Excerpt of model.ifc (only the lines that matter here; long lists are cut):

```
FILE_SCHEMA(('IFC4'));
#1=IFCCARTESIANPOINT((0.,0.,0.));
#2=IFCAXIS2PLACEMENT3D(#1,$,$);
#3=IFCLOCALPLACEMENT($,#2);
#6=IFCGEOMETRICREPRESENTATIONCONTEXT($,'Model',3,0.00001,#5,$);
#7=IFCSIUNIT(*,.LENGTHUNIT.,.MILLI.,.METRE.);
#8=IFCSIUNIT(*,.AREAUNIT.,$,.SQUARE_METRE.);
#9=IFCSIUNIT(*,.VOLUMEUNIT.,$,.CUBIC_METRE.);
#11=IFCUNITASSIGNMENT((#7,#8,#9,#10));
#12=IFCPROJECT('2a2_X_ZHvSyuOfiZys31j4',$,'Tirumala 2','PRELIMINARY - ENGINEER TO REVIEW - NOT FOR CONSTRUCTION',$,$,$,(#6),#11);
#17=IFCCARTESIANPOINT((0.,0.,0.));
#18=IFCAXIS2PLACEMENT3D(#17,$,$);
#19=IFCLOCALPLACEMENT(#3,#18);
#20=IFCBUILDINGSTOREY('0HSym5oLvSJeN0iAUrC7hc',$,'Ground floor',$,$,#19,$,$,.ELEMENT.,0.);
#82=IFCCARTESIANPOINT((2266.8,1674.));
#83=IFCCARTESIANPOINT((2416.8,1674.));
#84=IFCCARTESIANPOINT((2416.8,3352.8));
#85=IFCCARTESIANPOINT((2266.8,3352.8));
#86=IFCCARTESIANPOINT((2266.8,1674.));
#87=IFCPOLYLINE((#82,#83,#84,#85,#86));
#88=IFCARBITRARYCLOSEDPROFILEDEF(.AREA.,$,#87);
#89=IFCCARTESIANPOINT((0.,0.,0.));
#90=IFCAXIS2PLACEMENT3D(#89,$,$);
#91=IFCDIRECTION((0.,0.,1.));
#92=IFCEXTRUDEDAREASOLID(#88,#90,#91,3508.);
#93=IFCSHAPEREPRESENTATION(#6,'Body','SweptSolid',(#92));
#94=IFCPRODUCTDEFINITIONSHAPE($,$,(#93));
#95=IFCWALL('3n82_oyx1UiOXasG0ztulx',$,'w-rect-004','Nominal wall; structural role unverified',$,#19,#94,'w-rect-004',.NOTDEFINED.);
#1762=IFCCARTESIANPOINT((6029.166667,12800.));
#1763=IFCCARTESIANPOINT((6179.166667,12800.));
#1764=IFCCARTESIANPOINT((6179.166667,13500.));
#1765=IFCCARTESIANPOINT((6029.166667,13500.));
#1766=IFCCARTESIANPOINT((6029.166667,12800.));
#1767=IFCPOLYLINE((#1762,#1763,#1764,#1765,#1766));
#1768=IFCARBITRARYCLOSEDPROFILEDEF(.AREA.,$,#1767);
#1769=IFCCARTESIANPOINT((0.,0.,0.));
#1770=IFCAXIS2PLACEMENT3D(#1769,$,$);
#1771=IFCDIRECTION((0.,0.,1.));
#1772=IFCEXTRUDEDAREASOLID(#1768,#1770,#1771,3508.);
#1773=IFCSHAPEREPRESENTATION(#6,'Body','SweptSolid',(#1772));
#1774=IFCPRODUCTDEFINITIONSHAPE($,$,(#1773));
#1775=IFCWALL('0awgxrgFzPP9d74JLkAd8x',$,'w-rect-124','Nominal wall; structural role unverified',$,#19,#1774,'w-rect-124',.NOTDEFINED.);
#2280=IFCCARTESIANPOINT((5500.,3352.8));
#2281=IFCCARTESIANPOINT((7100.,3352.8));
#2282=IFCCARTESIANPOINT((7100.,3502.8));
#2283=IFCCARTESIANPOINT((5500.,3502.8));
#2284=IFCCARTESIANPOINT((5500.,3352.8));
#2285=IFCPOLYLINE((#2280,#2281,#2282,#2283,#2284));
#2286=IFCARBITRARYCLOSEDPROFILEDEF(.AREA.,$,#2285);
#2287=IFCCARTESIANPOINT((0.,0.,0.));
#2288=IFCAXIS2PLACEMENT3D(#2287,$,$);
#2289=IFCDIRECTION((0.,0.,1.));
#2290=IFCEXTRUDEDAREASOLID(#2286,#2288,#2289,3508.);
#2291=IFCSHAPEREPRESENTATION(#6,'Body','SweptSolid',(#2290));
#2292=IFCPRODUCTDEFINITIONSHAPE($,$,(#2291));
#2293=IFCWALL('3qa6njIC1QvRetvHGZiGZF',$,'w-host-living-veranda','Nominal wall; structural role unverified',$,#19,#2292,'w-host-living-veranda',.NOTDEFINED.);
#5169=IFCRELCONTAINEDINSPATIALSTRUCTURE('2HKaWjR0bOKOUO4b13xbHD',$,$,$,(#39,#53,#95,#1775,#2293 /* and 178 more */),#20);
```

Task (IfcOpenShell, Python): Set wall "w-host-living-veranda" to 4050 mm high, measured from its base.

```python
import ifcopenshell
import ifcopenshell.geom
import ifcopenshell.util.shape

model = ifcopenshell.open("model.ifc")
settings = ifcopenshell.geom.settings()


def volume(element):
    """Net volume in cubic metres, openings subtracted."""
    shape = ifcopenshell.geom.create_shape(settings, element)
    return ifcopenshell.util.shape.get_volume(shape.geometry)


wall = model.by_guid("3qa6njIC1QvRetvHGZiGZF")
before = volume(wall)

body = next(r for r in wall.Representation.Representations if r.RepresentationIdentifier == "Body")
solid = body.Items[0]
old_height = solid.Depth
solid.Depth = 4050.0
after = volume(wall)

print(f"height {old_height:g} -> {solid.Depth:g}, volume {before:.3f} -> {after:.3f} m3")

model.write("model_edited.ifc")
```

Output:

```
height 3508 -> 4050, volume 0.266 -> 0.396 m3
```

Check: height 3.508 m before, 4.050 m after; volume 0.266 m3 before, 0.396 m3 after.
